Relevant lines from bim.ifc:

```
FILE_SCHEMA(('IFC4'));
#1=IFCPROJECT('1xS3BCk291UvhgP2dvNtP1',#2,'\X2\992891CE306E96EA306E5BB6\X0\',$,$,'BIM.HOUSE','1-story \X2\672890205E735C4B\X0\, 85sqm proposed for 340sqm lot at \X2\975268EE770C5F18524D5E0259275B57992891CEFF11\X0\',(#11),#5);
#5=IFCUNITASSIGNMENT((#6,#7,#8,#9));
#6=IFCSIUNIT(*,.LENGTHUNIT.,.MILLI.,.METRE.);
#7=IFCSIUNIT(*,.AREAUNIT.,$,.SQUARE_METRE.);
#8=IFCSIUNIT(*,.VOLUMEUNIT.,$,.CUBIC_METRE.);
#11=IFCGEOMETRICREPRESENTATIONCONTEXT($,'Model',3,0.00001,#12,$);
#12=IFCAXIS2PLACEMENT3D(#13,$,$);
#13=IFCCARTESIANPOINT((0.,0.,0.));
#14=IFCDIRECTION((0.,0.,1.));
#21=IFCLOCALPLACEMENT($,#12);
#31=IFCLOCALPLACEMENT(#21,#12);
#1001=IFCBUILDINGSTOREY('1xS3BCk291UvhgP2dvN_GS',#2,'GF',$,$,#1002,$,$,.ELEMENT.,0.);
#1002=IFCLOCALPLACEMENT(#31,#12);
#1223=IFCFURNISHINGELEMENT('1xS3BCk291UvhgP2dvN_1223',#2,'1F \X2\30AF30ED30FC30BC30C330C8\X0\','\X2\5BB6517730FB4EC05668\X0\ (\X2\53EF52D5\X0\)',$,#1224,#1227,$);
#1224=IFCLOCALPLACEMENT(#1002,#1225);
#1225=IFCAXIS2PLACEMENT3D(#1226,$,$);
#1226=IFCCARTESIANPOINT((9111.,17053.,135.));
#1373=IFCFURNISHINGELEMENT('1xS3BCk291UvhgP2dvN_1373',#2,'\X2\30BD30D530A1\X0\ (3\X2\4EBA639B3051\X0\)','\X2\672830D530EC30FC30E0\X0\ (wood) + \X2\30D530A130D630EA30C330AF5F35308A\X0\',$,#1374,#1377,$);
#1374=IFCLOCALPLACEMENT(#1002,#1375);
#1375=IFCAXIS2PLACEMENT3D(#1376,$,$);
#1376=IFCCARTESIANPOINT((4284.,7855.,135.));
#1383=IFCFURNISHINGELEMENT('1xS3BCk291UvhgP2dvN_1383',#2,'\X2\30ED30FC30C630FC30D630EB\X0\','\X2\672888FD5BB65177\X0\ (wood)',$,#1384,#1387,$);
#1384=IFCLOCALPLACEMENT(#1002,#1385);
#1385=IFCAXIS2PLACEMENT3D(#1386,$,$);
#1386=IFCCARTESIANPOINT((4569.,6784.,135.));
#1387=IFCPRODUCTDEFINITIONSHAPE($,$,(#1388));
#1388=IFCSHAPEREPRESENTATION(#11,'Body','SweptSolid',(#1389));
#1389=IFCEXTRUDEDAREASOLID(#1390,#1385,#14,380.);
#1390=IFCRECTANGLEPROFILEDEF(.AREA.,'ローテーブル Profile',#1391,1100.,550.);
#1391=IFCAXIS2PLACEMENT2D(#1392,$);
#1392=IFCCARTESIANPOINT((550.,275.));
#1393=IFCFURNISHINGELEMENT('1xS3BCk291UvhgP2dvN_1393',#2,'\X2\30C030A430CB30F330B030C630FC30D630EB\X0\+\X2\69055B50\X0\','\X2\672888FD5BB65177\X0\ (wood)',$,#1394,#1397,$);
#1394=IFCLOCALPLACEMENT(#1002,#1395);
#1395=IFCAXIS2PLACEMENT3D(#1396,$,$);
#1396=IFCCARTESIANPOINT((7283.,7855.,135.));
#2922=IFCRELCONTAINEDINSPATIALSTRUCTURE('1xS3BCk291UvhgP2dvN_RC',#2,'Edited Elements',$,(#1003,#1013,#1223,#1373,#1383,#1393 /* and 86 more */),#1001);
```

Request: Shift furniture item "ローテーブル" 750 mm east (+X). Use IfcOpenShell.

```python
import ifcopenshell
import ifcopenshell.api.geometry
import ifcopenshell.util.placement

model = ifcopenshell.open("bim.ifc")

item = model.by_guid("1xS3BCk291UvhgP2dvN_1383")
matrix = ifcopenshell.util.placement.get_local_placement(item.ObjectPlacement)
matrix[0, 3] += 750.0
ifcopenshell.api.geometry.edit_object_placement(model, product=item, matrix=matrix, is_si=False)

print(ifcopenshell.util.placement.get_local_placement(item.ObjectPlacement).round(3) + 0.0)

model.write("bim_v2.ifc")
```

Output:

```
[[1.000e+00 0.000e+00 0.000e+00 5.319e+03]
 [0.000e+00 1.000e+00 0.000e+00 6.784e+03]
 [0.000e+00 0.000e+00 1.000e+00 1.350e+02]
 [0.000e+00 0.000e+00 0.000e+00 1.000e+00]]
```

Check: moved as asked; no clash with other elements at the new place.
